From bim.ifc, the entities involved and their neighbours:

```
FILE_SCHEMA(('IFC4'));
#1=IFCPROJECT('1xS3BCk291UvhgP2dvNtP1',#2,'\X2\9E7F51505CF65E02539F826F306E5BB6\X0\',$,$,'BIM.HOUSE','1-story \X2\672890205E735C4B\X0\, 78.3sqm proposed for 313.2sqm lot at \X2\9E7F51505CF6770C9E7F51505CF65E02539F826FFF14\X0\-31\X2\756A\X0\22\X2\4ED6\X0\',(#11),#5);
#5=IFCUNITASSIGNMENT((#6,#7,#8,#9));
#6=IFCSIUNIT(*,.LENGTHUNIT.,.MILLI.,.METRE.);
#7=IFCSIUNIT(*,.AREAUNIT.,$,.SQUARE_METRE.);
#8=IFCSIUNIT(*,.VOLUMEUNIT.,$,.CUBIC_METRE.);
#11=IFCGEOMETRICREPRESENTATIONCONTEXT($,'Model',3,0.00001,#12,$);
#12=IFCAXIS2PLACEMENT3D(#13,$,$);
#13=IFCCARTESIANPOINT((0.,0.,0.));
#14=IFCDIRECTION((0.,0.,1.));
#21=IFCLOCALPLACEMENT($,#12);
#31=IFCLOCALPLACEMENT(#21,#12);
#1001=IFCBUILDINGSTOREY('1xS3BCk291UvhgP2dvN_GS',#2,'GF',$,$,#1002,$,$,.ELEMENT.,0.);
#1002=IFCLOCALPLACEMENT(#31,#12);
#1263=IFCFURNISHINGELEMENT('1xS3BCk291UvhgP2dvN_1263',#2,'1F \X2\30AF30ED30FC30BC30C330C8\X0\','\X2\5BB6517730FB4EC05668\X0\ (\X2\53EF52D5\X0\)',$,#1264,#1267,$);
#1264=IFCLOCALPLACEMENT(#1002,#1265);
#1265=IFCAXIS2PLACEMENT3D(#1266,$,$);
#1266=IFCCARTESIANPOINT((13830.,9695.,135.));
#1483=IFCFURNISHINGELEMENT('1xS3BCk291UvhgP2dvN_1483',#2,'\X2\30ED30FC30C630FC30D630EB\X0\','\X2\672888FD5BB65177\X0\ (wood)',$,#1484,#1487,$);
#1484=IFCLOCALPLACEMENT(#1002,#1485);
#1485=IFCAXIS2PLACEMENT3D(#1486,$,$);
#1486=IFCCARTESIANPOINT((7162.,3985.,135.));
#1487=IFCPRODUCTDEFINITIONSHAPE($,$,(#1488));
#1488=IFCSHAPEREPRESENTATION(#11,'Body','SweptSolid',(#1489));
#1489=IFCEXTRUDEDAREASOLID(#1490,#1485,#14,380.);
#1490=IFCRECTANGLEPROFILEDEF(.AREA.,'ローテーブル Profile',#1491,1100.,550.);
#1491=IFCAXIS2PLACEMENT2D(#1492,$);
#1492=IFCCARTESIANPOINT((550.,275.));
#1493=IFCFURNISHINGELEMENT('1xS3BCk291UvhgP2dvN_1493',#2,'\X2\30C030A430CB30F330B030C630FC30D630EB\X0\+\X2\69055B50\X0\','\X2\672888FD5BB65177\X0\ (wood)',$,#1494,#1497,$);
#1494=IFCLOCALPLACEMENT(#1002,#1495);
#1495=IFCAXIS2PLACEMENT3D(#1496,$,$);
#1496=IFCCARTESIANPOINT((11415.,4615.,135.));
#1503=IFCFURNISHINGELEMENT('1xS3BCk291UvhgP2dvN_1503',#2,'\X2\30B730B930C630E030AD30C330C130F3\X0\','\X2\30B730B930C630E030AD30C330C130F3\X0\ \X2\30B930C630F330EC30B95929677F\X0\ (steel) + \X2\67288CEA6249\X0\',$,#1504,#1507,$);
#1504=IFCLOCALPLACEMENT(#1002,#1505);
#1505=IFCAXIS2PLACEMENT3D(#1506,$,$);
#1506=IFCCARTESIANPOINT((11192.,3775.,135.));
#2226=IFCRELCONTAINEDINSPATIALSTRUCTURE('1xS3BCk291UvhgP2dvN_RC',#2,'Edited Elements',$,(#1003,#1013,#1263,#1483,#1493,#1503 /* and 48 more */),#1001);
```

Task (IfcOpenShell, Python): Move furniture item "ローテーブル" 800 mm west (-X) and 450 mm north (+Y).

```python
import ifcopenshell
import ifcopenshell.api.geometry
import ifcopenshell.util.placement
import ifcopenshell.util.unit

model = ifcopenshell.open("bim.ifc")
unit_scale = ifcopenshell.util.unit.calculate_unit_scale(model)

item = model.by_guid("1xS3BCk291UvhgP2dvN_1483")
matrix = ifcopenshell.util.placement.get_local_placement(item.ObjectPlacement)
matrix[0, 3] -= 0.8 / unit_scale
matrix[1, 3] += 0.45 / unit_scale
ifcopenshell.api.geometry.edit_object_placement(model, product=item, matrix=matrix, is_si=False)

print(ifcopenshell.util.placement.get_local_placement(item.ObjectPlacement).round(3) + 0.0)

model.write("bim_edited.ifc")
```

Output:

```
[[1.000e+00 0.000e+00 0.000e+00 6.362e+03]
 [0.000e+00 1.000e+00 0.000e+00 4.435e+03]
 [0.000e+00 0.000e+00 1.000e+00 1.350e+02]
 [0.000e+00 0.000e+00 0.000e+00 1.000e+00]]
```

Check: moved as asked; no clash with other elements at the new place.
